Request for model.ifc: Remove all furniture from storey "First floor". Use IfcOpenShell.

First a look at what the model holds.

```python
import ifcopenshell
import ifcopenshell.util.element

model = ifcopenshell.open("model.ifc")
print(model.schema)
storey = next(s for s in model.by_type("IfcBuildingStorey") if s.Name == "First floor")
furniture = [e for e in ifcopenshell.util.element.get_decomposition(storey) if e.is_a("IfcFurnishingElement")]
seen = {}
for e in furniture:
    element_type = ifcopenshell.util.element.get_type(e)
    name = element_type.Name if element_type not in (None, e) else None
    seen[name] = seen.get(name, 0) + 1
for name, count in sorted(seen.items(), key=str):
    print(count, "x", name)
```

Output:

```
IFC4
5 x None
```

```python
import ifcopenshell
import ifcopenshell.api.root
import ifcopenshell.util.element

model = ifcopenshell.open("model.ifc")

storey = next(s for s in model.by_type("IfcBuildingStorey") if s.Name == "First floor")
furniture = [e for e in ifcopenshell.util.element.get_decomposition(storey) if e.is_a("IfcFurnishingElement")]

for e in furniture:
    ifcopenshell.api.root.remove_product(model, product=e)
print(len(furniture), "removed")

model.write("model_rev.ifc")
```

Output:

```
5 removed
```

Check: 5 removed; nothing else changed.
